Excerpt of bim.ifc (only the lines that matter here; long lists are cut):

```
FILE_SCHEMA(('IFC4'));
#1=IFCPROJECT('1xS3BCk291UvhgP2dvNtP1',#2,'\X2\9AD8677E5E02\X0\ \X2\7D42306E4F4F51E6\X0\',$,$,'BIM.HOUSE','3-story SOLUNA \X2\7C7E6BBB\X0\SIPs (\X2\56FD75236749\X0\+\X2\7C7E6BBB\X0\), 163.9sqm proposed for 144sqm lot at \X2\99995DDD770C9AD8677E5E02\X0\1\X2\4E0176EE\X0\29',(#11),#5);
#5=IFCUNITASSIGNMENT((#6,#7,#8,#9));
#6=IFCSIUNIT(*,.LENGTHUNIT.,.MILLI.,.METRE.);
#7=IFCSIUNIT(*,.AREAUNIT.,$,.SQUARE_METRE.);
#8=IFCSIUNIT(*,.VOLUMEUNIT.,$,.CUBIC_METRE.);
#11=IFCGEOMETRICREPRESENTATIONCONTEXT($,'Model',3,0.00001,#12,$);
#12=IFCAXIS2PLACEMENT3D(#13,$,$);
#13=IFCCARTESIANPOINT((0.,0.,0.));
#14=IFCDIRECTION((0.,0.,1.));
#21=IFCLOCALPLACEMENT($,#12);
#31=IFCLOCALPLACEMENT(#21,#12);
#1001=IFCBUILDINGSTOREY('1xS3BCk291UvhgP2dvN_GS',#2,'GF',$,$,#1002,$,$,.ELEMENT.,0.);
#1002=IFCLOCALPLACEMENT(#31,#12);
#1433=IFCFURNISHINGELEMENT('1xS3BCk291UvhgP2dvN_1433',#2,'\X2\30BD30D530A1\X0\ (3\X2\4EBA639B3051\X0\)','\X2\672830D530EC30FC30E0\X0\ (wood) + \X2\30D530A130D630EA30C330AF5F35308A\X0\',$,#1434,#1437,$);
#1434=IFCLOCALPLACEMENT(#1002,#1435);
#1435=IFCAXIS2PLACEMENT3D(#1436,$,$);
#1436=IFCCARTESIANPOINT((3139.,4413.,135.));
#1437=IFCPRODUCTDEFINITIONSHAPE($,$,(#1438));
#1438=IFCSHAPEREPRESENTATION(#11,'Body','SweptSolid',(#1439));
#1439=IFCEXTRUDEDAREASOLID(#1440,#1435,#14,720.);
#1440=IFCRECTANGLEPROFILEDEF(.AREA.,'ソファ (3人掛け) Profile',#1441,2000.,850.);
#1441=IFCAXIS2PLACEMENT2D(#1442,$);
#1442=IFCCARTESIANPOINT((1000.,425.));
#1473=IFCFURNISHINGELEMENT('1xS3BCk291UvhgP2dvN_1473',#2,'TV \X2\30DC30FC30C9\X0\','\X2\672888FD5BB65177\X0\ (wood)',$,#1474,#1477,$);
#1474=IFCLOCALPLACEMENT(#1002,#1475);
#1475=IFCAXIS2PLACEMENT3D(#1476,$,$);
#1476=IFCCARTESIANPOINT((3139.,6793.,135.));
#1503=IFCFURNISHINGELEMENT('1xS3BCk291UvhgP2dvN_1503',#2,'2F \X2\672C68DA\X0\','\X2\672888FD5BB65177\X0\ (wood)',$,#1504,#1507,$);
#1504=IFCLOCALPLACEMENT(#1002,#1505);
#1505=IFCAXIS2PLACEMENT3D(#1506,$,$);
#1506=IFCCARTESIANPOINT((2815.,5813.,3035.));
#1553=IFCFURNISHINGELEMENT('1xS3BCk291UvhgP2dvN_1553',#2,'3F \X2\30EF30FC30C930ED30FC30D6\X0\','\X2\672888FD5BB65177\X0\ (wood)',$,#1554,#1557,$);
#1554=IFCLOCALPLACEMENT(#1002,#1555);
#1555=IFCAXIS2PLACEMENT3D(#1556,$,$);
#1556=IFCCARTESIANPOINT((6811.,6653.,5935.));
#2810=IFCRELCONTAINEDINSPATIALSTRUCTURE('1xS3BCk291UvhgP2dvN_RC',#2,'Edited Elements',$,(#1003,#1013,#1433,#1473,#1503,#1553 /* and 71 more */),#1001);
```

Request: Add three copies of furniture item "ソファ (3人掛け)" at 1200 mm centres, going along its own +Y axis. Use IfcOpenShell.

```python
import ifcopenshell
import ifcopenshell.api.geometry
import ifcopenshell.api.root
import ifcopenshell.util.element
import ifcopenshell.util.placement
import ifcopenshell.util.unit

model = ifcopenshell.open("bim.ifc")
unit_scale = ifcopenshell.util.unit.calculate_unit_scale(model)


def reuse_history(source, copy):
    """copy_class also copies each property set's owner history, people and application; keep the originals."""
    for rel in copy.IsDefinedBy:
        if rel.is_a("IfcRelDefinesByProperties") and (history := rel.RelatingPropertyDefinition.OwnerHistory):
            rel.RelatingPropertyDefinition.OwnerHistory = source.OwnerHistory
            ifcopenshell.util.element.remove_deep2(model, history)


source = model.by_id(1433)
base = ifcopenshell.util.placement.get_local_placement(source.ObjectPlacement)
step = base[:3, 1] * 1.2 / unit_scale

for i in range(1, 4):
    copy = ifcopenshell.api.root.copy_class(model, product=source)
    copy.Representation = ifcopenshell.util.element.copy_deep(
        model, source.Representation, exclude=["IfcGeometricRepresentationContext", "IfcRepresentationMap"]
    )
    reuse_history(source, copy)
    matrix = base.copy()
    matrix[:3, 3] += i * step
    print("added at", matrix[:3, 3].round(3) + 0.0)
    ifcopenshell.api.geometry.edit_object_placement(model, product=copy, matrix=matrix, is_si=False)

model.write("bim_edited.ifc")
```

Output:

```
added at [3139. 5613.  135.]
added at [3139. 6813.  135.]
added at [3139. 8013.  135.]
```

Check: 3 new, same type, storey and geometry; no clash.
